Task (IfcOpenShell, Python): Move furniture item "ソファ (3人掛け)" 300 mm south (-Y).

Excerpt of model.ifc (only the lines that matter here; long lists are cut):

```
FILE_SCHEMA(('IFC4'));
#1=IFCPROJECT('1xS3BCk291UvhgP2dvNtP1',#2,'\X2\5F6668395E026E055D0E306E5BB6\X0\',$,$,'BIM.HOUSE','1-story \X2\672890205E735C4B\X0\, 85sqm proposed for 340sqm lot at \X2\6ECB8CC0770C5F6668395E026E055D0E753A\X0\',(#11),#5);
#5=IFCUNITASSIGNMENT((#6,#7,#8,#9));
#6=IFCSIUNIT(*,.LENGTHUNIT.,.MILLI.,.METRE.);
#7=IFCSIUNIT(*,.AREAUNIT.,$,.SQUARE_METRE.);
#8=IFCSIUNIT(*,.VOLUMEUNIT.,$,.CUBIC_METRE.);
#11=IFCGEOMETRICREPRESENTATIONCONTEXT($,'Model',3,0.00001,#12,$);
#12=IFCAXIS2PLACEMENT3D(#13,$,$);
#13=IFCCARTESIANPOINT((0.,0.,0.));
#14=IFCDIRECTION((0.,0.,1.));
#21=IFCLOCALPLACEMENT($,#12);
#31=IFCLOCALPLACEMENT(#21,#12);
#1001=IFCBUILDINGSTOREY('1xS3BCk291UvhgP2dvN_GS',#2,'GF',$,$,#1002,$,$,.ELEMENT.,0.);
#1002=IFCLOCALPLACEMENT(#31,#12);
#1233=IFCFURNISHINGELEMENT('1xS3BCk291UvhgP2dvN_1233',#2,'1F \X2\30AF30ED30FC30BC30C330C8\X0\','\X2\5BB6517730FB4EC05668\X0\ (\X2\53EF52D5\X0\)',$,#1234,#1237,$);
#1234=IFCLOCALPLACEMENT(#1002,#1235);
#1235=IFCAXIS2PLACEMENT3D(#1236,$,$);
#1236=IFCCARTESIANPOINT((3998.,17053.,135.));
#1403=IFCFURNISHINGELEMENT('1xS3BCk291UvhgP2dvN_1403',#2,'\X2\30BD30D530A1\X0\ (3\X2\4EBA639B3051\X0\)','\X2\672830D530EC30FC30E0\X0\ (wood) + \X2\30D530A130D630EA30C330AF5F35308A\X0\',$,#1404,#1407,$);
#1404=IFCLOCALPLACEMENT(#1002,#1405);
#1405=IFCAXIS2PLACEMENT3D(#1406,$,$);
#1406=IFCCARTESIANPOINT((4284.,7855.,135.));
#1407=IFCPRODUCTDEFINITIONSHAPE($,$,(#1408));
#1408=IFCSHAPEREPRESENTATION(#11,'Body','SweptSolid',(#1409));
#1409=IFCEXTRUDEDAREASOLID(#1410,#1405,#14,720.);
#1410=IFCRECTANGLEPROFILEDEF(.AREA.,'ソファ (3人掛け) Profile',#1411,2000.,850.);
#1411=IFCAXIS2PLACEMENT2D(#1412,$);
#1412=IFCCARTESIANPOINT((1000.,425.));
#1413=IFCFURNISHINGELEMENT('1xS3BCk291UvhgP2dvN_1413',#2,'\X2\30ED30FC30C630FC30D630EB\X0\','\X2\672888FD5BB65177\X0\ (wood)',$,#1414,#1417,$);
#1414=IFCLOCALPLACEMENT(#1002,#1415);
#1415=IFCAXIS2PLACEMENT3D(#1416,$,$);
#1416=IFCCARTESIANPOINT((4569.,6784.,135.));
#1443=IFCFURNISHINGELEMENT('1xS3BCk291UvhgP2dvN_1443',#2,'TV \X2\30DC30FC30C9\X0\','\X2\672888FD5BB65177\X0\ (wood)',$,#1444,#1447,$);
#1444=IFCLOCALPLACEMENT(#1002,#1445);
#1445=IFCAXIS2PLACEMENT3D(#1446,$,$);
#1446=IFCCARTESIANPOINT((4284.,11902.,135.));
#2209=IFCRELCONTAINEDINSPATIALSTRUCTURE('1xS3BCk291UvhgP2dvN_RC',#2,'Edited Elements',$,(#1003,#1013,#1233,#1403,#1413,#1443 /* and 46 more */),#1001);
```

```python
import ifcopenshell
import ifcopenshell.api.geometry
import ifcopenshell.util.placement

model = ifcopenshell.open("model.ifc")

item = model.by_id(1403)
matrix = ifcopenshell.util.placement.get_local_placement(item.ObjectPlacement)
matrix[1, 3] -= 300.0
ifcopenshell.api.geometry.edit_object_placement(model, product=item, matrix=matrix, is_si=False)

print(ifcopenshell.util.placement.get_local_placement(item.ObjectPlacement).round(3) + 0.0)

model.write("model_edited.ifc")
```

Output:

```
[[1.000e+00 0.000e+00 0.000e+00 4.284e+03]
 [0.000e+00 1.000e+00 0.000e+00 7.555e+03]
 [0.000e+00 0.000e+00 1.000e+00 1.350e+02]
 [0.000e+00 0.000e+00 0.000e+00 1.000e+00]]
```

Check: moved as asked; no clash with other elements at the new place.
